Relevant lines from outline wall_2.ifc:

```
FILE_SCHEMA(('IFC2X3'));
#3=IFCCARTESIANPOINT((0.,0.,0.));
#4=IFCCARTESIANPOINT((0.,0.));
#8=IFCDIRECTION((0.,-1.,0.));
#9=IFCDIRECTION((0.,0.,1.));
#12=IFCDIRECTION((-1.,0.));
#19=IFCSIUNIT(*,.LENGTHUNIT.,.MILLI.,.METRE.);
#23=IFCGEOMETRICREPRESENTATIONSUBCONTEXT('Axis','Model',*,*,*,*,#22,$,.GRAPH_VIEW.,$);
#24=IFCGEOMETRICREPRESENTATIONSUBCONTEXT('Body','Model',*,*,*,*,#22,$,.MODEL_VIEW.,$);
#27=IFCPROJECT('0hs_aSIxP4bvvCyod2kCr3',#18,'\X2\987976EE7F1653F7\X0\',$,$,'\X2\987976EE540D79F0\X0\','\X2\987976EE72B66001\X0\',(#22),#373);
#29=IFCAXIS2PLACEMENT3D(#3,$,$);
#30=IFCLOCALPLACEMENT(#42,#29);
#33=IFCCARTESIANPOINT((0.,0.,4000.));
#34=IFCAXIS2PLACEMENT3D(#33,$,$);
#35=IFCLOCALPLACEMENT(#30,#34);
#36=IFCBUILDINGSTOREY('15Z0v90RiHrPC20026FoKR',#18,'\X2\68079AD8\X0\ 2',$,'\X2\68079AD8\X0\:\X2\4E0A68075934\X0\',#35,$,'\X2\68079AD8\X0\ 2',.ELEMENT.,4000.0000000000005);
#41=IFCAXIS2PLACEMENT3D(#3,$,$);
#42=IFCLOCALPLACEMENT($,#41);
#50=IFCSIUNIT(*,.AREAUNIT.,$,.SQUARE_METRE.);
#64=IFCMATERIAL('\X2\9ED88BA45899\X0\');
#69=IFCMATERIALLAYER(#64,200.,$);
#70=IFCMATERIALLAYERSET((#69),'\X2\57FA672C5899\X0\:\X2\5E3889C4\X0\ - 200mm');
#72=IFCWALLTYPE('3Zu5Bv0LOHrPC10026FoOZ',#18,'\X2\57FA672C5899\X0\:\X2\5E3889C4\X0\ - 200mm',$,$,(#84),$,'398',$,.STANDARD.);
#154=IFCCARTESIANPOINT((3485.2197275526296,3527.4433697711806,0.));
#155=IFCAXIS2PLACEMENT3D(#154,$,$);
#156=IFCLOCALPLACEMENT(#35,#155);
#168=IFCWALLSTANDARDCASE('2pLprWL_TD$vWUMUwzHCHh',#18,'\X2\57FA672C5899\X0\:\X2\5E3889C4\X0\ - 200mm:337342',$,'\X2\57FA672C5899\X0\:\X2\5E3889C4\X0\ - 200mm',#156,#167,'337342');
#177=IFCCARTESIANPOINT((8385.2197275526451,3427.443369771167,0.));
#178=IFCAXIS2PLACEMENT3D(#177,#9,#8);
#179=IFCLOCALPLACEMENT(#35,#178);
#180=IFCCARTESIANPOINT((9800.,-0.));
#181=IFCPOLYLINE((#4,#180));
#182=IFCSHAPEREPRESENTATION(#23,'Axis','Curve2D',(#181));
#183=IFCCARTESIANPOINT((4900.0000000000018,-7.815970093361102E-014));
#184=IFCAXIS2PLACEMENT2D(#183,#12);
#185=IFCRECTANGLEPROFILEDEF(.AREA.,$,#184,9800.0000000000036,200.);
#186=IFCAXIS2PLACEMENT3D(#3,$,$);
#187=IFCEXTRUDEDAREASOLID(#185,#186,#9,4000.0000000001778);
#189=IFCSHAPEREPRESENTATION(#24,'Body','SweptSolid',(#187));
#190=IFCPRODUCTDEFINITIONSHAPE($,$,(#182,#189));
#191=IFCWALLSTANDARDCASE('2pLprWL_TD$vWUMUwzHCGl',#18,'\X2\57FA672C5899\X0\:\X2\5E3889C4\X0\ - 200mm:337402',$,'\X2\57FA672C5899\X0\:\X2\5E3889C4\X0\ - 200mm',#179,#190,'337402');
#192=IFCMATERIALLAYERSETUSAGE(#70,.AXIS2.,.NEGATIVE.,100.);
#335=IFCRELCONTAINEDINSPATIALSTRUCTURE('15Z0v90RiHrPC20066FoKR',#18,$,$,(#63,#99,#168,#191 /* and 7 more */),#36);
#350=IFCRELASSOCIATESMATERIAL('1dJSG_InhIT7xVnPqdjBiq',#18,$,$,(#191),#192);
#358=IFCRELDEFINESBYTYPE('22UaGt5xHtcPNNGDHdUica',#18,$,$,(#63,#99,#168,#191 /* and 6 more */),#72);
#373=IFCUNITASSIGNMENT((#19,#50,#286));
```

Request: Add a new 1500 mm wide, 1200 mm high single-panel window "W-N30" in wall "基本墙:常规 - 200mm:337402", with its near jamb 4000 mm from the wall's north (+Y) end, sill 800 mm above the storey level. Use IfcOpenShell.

```python
import numpy as np
import ifcopenshell
import ifcopenshell.api.feature
import ifcopenshell.api.geometry
import ifcopenshell.api.root
import ifcopenshell.api.spatial
import ifcopenshell.api.type
import ifcopenshell.geom
import ifcopenshell.util.element
import ifcopenshell.util.placement
import ifcopenshell.util.representation
import ifcopenshell.util.shape
import ifcopenshell.util.unit

model = ifcopenshell.open("outline wall_2.ifc")
unit_scale = ifcopenshell.util.unit.calculate_unit_scale(model)
settings = ifcopenshell.geom.settings()


def volume(element):
    """Net volume in cubic metres, openings subtracted."""
    shape = ifcopenshell.geom.create_shape(settings, element)
    return ifcopenshell.util.shape.get_volume(shape.geometry)


wall = model.by_guid("2pLprWL_TD$vWUMUwzHCGl")
storey = ifcopenshell.util.element.get_container(wall, ifc_class="IfcBuildingStorey")
context = ifcopenshell.util.representation.get_context(model, "Model", "Body", "MODEL_VIEW")
before = volume(wall)

width, height, from_end, sill = 1.5, 1.2, 4, 0.8  # metres

# The wall runs along its own X axis, and the end named is its -X end.
wall_shape = ifcopenshell.geom.create_shape(settings, wall)
x, y, z = ifcopenshell.util.shape.get_vertices(wall_shape.geometry).T
start = x.min() + from_end
face, thickness = float(y.min()), float(y.max() - y.min())
wall_matrix = ifcopenshell.util.placement.get_local_placement(wall.ObjectPlacement)
level = ifcopenshell.util.placement.get_local_placement(storey.ObjectPlacement)[2, 3]


def in_wall(x, y):
    """Placement at x, y metres in the wall's axes, at sill height."""
    matrix = wall_matrix.copy()
    matrix[:, 3] = wall_matrix @ np.array([x / unit_scale, y / unit_scale, 0.0, 1.0])
    matrix[2, 3] = level + sill / unit_scale
    return matrix


# Opening: a box that overshoots both wall faces by 50 mm.
opening = ifcopenshell.api.root.create_entity(model, ifc_class="IfcOpeningElement")
box = ifcopenshell.api.geometry.add_wall_representation(
    model, context=context, length=width, height=height, thickness=thickness + 0.1
)
ifcopenshell.api.geometry.assign_representation(model, product=opening, representation=box)
ifcopenshell.api.geometry.edit_object_placement(model, product=opening, matrix=in_wall(start, face - 0.05), is_si=False)
ifcopenshell.api.feature.add_feature(model, feature=opening, element=wall)

window = ifcopenshell.api.root.create_entity(model, ifc_class="IfcWindow", name="W-N30")
window.OverallWidth, window.OverallHeight = width / unit_scale, height / unit_scale
body = ifcopenshell.api.geometry.add_window_representation(
    model,
    context=context,
    overall_width=window.OverallWidth,
    overall_height=window.OverallHeight,
    partition_type="SINGLE_PANEL",
)
ifcopenshell.api.geometry.assign_representation(model, product=window, representation=body)
ifcopenshell.api.spatial.assign_container(model, products=[window], relating_structure=storey)
fills = ifcopenshell.api.feature.add_filling(model, opening=opening, element=window)
fills.OwnerHistory = window.OwnerHistory  # required in IFC2X3

# IFC2X3 keeps the operation on the window style.
style = ifcopenshell.api.root.create_entity(model, ifc_class="IfcWindowStyle", name="W-N30")
style.OperationType, style.ConstructionType = "SINGLE_PANEL", "NOTDEFINED"
style.ParameterTakesPrecedence = style.Sizeable = False
ifcopenshell.api.type.assign_type(model, related_objects=[window], relating_type=style)

# Centre the window in the wall's thickness.
ifcopenshell.api.geometry.edit_object_placement(model, product=window, matrix=in_wall(start, face), is_si=False)
window_shape = ifcopenshell.geom.create_shape(settings, window)
depth = ifcopenshell.util.shape.get_vertices(window_shape.geometry)[:, 1]
offset = face + thickness / 2 - (depth.min() + depth.max()) / 2
ifcopenshell.api.geometry.edit_object_placement(model, product=window, matrix=in_wall(start, offset), is_si=False)

after = volume(wall)

print(f"wall volume {before:.3f} -> {after:.3f} m3")

model.write("outline wall_2_v2.ifc")
```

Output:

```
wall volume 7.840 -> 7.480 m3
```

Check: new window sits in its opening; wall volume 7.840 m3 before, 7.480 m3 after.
